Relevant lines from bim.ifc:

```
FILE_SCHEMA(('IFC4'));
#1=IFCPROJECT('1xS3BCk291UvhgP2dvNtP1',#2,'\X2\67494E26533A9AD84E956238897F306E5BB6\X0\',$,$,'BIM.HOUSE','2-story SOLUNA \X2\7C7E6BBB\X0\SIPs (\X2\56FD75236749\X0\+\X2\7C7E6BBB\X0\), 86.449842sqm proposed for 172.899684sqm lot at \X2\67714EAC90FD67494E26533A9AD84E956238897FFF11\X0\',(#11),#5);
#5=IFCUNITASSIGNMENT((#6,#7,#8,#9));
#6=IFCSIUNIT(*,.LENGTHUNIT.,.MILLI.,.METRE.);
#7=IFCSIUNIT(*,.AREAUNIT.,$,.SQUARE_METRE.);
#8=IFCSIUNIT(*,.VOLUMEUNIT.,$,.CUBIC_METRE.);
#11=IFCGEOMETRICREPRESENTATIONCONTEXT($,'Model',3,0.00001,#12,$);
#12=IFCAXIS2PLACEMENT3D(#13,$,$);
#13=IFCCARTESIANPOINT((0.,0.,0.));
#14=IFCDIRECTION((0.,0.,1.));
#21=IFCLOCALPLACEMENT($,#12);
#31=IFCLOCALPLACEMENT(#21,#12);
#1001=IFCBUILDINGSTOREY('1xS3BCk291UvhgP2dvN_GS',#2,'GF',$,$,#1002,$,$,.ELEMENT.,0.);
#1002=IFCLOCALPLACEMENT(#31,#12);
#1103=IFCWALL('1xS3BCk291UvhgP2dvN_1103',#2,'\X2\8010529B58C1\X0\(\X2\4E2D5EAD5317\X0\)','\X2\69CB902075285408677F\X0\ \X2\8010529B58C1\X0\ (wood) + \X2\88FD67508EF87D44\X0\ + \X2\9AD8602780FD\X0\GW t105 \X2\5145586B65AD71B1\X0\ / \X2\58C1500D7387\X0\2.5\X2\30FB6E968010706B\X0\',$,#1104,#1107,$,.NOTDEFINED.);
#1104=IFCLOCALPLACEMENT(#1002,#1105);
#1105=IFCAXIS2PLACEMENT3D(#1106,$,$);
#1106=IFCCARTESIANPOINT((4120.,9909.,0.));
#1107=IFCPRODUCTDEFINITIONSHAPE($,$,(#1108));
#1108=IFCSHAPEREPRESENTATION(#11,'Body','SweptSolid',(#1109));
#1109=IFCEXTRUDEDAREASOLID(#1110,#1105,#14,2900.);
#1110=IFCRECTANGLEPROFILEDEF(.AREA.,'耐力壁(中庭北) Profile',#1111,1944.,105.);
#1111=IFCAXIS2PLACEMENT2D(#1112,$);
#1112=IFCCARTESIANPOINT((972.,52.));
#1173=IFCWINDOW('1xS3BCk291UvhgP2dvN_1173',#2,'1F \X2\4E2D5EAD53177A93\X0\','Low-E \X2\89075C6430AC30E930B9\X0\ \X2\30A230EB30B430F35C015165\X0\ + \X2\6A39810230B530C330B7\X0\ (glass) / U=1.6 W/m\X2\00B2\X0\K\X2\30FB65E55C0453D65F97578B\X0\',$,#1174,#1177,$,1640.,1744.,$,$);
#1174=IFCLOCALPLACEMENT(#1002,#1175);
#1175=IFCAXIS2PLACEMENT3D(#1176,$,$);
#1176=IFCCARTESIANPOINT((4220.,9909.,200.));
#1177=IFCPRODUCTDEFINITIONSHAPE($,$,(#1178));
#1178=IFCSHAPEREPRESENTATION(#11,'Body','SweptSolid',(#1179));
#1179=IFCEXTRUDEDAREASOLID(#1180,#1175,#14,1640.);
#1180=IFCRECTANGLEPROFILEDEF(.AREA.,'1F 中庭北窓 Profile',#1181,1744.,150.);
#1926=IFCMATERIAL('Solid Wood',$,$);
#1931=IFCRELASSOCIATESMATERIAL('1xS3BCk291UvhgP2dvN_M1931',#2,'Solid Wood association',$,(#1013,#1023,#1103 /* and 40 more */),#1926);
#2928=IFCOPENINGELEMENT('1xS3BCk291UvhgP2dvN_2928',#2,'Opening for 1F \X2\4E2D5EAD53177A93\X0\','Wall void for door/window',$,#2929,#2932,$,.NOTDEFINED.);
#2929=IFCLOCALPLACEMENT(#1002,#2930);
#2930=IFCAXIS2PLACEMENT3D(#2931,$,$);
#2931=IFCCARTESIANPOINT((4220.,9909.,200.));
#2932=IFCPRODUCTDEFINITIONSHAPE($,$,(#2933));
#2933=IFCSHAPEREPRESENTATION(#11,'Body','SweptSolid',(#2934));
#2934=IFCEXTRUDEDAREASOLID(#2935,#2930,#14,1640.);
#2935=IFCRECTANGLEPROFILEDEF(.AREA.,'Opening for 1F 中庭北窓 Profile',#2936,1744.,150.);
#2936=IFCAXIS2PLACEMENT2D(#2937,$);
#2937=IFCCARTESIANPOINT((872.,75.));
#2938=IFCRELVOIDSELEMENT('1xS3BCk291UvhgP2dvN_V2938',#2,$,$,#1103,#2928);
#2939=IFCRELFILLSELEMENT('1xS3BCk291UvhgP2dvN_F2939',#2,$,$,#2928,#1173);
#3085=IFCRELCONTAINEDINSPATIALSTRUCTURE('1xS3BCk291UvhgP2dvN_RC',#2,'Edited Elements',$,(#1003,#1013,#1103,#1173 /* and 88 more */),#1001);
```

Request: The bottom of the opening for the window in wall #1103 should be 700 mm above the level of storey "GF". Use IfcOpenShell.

```python
import numpy as np
import ifcopenshell
import ifcopenshell.api.geometry
import ifcopenshell.geom
import ifcopenshell.util.element
import ifcopenshell.util.placement
import ifcopenshell.util.shape
import ifcopenshell.util.unit

model = ifcopenshell.open("bim.ifc")
unit_scale = ifcopenshell.util.unit.calculate_unit_scale(model)

window = model.by_guid("1xS3BCk291UvhgP2dvN_1173")
opening = window.FillsVoids[0].RelatingOpeningElement
storey = ifcopenshell.util.element.get_container(window, ifc_class="IfcBuildingStorey")
level = ifcopenshell.util.placement.get_local_placement(storey.ObjectPlacement)[2, 3]

# The opening's origin need not be at the sill, so measure its lowest point.
shape = ifcopenshell.geom.create_shape(ifcopenshell.geom.settings(), opening)
bottom = ifcopenshell.util.shape.get_shape_bottom_elevation(shape, shape.geometry) / unit_scale
dz = level + 700.0 - bottom

shift = np.array([0.0, 0.0, dz])
# The window is not placed relative to its opening, so move both.
for product in (opening, window):
    matrix = ifcopenshell.util.placement.get_local_placement(product.ObjectPlacement)
    matrix[:3, 3] += shift
    ifcopenshell.api.geometry.edit_object_placement(model, product=product, matrix=matrix, is_si=False)

print(f"moved by {dz * unit_scale:+.3f} m")

model.write("bim_rev.ifc")
```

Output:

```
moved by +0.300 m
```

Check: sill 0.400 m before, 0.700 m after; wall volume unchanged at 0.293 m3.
